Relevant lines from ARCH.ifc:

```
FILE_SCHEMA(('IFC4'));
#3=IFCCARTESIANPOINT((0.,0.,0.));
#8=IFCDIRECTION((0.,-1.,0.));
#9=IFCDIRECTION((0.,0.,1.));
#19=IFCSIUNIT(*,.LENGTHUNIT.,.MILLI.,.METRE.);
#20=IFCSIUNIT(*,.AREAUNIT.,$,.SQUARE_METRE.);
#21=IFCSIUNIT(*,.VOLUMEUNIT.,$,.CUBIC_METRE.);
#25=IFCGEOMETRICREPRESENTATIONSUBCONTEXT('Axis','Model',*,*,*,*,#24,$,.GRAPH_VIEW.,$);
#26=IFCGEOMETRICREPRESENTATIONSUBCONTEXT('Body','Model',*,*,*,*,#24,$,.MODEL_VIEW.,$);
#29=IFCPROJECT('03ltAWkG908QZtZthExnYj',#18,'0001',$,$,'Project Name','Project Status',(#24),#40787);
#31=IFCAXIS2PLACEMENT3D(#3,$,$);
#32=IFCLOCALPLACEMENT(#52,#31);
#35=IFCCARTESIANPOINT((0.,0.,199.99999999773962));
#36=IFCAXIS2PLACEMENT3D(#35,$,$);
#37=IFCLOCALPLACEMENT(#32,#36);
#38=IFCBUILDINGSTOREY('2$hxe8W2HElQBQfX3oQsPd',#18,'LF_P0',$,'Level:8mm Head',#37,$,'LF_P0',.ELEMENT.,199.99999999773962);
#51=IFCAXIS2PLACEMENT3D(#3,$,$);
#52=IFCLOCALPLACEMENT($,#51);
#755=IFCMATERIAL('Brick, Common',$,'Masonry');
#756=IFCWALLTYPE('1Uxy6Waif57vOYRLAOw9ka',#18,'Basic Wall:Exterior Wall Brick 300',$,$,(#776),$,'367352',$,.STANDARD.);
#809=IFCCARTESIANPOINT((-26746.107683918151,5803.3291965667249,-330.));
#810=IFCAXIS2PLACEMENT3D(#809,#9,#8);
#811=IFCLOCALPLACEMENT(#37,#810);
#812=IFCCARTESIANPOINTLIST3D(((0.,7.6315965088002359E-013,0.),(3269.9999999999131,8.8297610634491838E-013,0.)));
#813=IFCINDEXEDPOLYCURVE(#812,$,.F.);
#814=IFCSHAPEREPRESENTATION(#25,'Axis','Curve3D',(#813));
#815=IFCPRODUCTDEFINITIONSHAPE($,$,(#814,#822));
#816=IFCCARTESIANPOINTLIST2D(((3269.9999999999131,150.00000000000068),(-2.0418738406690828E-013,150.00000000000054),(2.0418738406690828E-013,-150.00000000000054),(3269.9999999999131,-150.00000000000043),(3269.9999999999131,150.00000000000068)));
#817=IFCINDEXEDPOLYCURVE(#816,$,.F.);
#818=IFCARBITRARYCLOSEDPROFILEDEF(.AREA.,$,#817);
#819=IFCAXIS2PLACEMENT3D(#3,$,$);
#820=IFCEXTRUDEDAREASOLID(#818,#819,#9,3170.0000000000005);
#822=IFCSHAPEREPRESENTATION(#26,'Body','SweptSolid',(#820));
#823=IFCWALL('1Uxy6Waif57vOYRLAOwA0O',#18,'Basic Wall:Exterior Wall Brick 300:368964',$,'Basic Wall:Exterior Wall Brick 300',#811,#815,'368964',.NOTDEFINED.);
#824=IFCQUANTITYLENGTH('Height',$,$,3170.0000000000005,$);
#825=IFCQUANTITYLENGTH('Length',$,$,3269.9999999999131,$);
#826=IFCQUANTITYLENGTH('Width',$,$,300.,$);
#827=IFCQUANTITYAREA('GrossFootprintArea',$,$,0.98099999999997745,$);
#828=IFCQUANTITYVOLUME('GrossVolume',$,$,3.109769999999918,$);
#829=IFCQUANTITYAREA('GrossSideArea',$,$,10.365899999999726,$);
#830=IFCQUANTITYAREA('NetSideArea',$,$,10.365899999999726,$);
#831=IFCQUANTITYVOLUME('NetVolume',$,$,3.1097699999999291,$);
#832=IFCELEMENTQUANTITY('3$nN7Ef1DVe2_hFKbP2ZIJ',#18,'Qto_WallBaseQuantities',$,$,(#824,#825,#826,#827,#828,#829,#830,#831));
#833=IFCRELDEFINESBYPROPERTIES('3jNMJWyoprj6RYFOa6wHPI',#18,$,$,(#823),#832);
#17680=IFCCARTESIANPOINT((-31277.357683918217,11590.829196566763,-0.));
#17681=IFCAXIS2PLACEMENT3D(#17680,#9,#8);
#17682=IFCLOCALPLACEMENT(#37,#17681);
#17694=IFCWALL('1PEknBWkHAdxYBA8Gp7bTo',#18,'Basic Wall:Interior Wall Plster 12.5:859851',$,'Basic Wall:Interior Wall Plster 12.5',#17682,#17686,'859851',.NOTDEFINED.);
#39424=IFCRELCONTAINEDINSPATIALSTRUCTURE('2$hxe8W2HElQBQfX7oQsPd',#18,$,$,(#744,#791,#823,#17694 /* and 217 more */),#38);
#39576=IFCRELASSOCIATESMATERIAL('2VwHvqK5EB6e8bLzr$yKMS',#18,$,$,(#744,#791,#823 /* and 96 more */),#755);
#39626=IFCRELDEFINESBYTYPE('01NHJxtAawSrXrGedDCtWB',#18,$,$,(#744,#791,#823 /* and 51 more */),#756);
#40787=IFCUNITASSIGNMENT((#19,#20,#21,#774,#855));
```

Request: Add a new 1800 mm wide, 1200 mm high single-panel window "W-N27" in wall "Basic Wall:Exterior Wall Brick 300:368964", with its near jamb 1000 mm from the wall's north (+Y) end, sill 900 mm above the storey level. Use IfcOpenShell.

```python
import numpy as np
import ifcopenshell
import ifcopenshell.api.feature
import ifcopenshell.api.geometry
import ifcopenshell.api.pset
import ifcopenshell.api.root
import ifcopenshell.api.spatial
import ifcopenshell.geom
import ifcopenshell.util.element
import ifcopenshell.util.placement
import ifcopenshell.util.representation
import ifcopenshell.util.shape
import ifcopenshell.util.unit

model = ifcopenshell.open("ARCH.ifc")
unit_scale = ifcopenshell.util.unit.calculate_unit_scale(model)
area_scale = ifcopenshell.util.unit.calculate_unit_scale(model, "AREAUNIT")
volume_scale = ifcopenshell.util.unit.calculate_unit_scale(model, "VOLUMEUNIT")
settings = ifcopenshell.geom.settings()


def volume(element):
    """Net volume in cubic metres, openings subtracted."""
    shape = ifcopenshell.geom.create_shape(settings, element)
    return ifcopenshell.util.shape.get_volume(shape.geometry)


wall = model.by_guid("1Uxy6Waif57vOYRLAOwA0O")
storey = ifcopenshell.util.element.get_container(wall, ifc_class="IfcBuildingStorey")
context = ifcopenshell.util.representation.get_context(model, "Model", "Body", "MODEL_VIEW")
before = volume(wall)

width, height, from_end, sill = 1.8, 1.2, 1, 0.9  # metres

# The wall runs along its own X axis, and the end named is its -X end.
wall_shape = ifcopenshell.geom.create_shape(settings, wall)
x, y, z = ifcopenshell.util.shape.get_vertices(wall_shape.geometry).T
start = x.min() + from_end
face, thickness = float(y.min()), float(y.max() - y.min())
wall_matrix = ifcopenshell.util.placement.get_local_placement(wall.ObjectPlacement)
level = ifcopenshell.util.placement.get_local_placement(storey.ObjectPlacement)[2, 3]


def in_wall(x, y):
    """Placement at x, y metres in the wall's axes, at sill height."""
    matrix = wall_matrix.copy()
    matrix[:, 3] = wall_matrix @ np.array([x / unit_scale, y / unit_scale, 0.0, 1.0])
    matrix[2, 3] = level + sill / unit_scale
    return matrix


# Opening: a box that overshoots both wall faces by 50 mm.
opening = ifcopenshell.api.root.create_entity(model, ifc_class="IfcOpeningElement", predefined_type="OPENING")
box = ifcopenshell.api.geometry.add_wall_representation(
    model, context=context, length=width, height=height, thickness=thickness + 0.1
)
ifcopenshell.api.geometry.assign_representation(model, product=opening, representation=box)
ifcopenshell.api.geometry.edit_object_placement(model, product=opening, matrix=in_wall(start, face - 0.05), is_si=False)
ifcopenshell.api.feature.add_feature(model, feature=opening, element=wall)

window = ifcopenshell.api.root.create_entity(model, ifc_class="IfcWindow", name="W-N27", predefined_type="WINDOW")
window.OverallWidth, window.OverallHeight = width / unit_scale, height / unit_scale
window.PartitioningType = "SINGLE_PANEL"
body = ifcopenshell.api.geometry.add_window_representation(
    model,
    context=context,
    overall_width=window.OverallWidth,
    overall_height=window.OverallHeight,
    partition_type="SINGLE_PANEL",
)
ifcopenshell.api.geometry.assign_representation(model, product=window, representation=body)
ifcopenshell.api.spatial.assign_container(model, products=[window], relating_structure=storey)
ifcopenshell.api.feature.add_filling(model, opening=opening, element=window)

# Centre the window in the wall's thickness.
ifcopenshell.api.geometry.edit_object_placement(model, product=window, matrix=in_wall(start, face), is_si=False)
window_shape = ifcopenshell.geom.create_shape(settings, window)
depth = ifcopenshell.util.shape.get_vertices(window_shape.geometry)[:, 1]
offset = face + thickness / 2 - (depth.min() + depth.max()) / 2
ifcopenshell.api.geometry.edit_object_placement(model, product=window, matrix=in_wall(start, offset), is_si=False)

after = volume(wall)

# Update the wall's stored quantities.
qto = model.by_id(ifcopenshell.util.element.get_pset(wall, "Qto_WallBaseQuantities", should_inherit=False)["id"])
ifcopenshell.api.pset.edit_qto(model, qto=qto, properties={
    "NetSideArea": after / thickness / area_scale,
    "NetVolume": after / volume_scale,
})

print(f"wall volume {before:.3f} -> {after:.3f} m3")

model.write("ARCH_updated.ifc")
```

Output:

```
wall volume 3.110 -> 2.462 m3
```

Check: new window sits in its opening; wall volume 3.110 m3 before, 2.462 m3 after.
